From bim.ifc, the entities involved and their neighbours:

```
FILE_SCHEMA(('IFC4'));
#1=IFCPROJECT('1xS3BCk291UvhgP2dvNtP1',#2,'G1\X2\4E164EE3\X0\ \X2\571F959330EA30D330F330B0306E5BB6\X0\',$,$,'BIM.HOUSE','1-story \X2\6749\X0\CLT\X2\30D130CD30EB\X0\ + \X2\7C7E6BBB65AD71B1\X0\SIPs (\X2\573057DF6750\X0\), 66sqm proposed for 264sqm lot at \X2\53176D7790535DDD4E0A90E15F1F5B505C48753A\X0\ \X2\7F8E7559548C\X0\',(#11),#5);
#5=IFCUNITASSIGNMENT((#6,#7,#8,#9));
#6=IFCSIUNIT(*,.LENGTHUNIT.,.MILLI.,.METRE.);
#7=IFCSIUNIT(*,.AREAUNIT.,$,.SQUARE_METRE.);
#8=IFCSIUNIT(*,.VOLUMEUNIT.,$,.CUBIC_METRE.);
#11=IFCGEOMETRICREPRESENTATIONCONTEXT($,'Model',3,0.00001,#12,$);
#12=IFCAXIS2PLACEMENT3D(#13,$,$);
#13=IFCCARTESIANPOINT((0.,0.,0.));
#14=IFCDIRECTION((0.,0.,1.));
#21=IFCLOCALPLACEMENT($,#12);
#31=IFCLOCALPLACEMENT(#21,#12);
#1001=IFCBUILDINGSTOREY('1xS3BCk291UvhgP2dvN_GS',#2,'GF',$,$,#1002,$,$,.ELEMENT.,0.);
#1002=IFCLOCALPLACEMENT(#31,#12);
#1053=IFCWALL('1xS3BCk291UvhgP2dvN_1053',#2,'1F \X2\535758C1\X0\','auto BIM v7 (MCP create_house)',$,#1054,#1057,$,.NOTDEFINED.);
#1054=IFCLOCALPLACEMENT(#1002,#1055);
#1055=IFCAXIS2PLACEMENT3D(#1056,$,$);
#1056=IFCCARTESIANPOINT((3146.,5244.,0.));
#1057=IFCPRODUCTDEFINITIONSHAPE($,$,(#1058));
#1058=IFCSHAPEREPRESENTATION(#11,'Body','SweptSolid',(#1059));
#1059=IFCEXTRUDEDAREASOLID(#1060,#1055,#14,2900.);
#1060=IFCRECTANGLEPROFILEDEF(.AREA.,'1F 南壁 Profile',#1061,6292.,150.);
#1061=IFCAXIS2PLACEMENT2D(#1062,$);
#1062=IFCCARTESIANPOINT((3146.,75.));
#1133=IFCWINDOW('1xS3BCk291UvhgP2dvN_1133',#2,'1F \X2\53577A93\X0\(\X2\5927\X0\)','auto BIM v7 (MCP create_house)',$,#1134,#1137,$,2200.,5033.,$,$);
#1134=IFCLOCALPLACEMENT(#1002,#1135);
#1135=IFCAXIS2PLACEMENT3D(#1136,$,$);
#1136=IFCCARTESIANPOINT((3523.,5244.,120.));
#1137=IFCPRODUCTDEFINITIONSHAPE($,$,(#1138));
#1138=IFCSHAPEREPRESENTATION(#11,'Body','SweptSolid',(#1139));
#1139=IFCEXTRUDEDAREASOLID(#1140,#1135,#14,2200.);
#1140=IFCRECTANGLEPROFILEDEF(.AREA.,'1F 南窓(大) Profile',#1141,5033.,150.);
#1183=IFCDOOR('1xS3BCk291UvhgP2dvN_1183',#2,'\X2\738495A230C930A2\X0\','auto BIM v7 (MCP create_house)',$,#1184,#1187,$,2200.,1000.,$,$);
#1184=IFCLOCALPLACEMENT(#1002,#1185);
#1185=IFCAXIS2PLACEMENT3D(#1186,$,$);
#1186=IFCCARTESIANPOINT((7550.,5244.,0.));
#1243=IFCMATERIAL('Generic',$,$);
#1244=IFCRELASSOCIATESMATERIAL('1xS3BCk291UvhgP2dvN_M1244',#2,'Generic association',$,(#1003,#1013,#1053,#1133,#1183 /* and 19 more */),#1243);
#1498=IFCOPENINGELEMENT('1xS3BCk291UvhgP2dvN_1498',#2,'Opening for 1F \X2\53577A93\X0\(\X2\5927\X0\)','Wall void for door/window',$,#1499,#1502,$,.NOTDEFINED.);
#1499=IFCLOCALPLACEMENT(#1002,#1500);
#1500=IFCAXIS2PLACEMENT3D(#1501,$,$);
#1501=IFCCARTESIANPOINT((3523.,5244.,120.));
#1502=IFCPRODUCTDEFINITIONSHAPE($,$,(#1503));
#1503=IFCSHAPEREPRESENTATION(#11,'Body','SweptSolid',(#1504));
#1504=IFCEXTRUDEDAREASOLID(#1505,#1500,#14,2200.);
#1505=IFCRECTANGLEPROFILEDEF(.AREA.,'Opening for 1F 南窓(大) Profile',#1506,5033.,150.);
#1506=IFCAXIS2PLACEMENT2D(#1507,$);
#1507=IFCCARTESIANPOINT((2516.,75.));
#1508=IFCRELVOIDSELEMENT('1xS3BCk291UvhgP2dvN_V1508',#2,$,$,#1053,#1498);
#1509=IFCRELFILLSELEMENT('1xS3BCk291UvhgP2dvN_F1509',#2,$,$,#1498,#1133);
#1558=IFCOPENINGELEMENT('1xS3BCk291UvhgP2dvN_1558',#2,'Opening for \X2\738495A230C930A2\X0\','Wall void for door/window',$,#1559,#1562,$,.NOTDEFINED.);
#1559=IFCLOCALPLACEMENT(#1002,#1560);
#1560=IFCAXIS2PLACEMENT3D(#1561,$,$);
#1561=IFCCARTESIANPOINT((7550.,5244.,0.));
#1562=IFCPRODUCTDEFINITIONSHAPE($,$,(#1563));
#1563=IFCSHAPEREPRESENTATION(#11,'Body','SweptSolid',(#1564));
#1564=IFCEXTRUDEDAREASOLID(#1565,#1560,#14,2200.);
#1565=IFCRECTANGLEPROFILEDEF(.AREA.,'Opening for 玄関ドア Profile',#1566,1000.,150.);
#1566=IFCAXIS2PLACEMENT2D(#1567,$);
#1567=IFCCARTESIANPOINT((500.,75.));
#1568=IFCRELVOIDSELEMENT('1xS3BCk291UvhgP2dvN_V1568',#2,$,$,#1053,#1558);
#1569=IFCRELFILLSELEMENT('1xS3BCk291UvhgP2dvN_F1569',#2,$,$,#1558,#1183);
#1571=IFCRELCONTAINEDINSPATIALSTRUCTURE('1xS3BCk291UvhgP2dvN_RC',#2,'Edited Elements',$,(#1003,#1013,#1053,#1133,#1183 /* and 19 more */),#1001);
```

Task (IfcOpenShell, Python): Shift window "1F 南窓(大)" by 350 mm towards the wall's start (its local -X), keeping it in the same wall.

```python
import ifcopenshell
import ifcopenshell.api.geometry
import ifcopenshell.util.placement

model = ifcopenshell.open("bim.ifc")

window = model.by_guid("1xS3BCk291UvhgP2dvN_1133")
opening = window.FillsVoids[0].RelatingOpeningElement
wall = opening.VoidsElements[0].RelatingBuildingElement

wall_matrix = ifcopenshell.util.placement.get_local_placement(wall.ObjectPlacement)
shift = wall_matrix[:3, 0] * -350.0
before = ifcopenshell.util.placement.get_local_placement(window.ObjectPlacement)[:3, 3].copy()

# The window is not placed relative to its opening, so move both.
for product in (opening, window):
    matrix = ifcopenshell.util.placement.get_local_placement(product.ObjectPlacement)
    matrix[:3, 3] += shift
    ifcopenshell.api.geometry.edit_object_placement(model, product=product, matrix=matrix, is_si=False)

after = ifcopenshell.util.placement.get_local_placement(window.ObjectPlacement)[:3, 3]
print("window moved by", (after - before).round(3) + 0.0)

model.write("bim_v2.ifc")
```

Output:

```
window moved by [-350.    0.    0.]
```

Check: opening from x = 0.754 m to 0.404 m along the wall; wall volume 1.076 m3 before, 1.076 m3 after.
